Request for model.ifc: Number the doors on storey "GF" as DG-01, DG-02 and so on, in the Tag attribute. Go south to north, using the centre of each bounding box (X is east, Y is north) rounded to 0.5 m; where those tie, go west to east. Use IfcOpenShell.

First a look at what the model holds.

```python
import ifcopenshell
import ifcopenshell.util.element
import ifcopenshell.util.placement

model = ifcopenshell.open("model.ifc")
print(model.schema)
storey = next(s for s in model.by_type("IfcBuildingStorey") if s.Name == "GF")
doors = [e for e in ifcopenshell.util.element.get_decomposition(storey) if e.is_a("IfcDoor")]
for e in sorted(doors, key=lambda e: e.id()):
    origin = ifcopenshell.util.placement.get_local_placement(e.ObjectPlacement)[:3, 3]
    print(e.id(), e.Tag, e.Name, origin.round(2) + 0.0, sep=" | ")
```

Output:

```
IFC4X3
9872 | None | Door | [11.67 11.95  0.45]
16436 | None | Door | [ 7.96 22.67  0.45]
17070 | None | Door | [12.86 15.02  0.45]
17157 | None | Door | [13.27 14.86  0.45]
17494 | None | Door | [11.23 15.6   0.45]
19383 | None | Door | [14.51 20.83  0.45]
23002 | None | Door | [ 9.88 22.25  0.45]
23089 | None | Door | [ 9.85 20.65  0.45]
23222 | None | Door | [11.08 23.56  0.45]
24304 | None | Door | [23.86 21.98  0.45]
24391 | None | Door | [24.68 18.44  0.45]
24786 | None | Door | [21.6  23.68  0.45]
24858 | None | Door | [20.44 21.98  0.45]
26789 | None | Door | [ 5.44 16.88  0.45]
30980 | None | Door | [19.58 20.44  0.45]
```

```python
import ifcopenshell
import ifcopenshell.geom
import ifcopenshell.util.element
import ifcopenshell.util.shape

model = ifcopenshell.open("model.ifc")
settings = ifcopenshell.geom.settings()
settings.set("use-world-coords", True)


def centre(element):
    shape = ifcopenshell.geom.create_shape(settings, element)
    return ifcopenshell.util.shape.get_bbox_centroid(shape.geometry)


storey = next(s for s in model.by_type("IfcBuildingStorey") if s.Name == "GF")
doors = [e for e in ifcopenshell.util.element.get_decomposition(storey) if e.is_a("IfcDoor")]

# Insertion points can sit at a corner or the storey origin, so sort by the geometry (in metres).
centres = {e: centre(e) for e in doors}
doors.sort(key=lambda e: (round(centres[e][1] / 0.5), centres[e][0]))

for i, e in enumerate(doors, start=1):
    number = f"DG-{i:02d}"
    e.Tag = number
    print(e.id(), number)

model.write("model_rev.ifc")
```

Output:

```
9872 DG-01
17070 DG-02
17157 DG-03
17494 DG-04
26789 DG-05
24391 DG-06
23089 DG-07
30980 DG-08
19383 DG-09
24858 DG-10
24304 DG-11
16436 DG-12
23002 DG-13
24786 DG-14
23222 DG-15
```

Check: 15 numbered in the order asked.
